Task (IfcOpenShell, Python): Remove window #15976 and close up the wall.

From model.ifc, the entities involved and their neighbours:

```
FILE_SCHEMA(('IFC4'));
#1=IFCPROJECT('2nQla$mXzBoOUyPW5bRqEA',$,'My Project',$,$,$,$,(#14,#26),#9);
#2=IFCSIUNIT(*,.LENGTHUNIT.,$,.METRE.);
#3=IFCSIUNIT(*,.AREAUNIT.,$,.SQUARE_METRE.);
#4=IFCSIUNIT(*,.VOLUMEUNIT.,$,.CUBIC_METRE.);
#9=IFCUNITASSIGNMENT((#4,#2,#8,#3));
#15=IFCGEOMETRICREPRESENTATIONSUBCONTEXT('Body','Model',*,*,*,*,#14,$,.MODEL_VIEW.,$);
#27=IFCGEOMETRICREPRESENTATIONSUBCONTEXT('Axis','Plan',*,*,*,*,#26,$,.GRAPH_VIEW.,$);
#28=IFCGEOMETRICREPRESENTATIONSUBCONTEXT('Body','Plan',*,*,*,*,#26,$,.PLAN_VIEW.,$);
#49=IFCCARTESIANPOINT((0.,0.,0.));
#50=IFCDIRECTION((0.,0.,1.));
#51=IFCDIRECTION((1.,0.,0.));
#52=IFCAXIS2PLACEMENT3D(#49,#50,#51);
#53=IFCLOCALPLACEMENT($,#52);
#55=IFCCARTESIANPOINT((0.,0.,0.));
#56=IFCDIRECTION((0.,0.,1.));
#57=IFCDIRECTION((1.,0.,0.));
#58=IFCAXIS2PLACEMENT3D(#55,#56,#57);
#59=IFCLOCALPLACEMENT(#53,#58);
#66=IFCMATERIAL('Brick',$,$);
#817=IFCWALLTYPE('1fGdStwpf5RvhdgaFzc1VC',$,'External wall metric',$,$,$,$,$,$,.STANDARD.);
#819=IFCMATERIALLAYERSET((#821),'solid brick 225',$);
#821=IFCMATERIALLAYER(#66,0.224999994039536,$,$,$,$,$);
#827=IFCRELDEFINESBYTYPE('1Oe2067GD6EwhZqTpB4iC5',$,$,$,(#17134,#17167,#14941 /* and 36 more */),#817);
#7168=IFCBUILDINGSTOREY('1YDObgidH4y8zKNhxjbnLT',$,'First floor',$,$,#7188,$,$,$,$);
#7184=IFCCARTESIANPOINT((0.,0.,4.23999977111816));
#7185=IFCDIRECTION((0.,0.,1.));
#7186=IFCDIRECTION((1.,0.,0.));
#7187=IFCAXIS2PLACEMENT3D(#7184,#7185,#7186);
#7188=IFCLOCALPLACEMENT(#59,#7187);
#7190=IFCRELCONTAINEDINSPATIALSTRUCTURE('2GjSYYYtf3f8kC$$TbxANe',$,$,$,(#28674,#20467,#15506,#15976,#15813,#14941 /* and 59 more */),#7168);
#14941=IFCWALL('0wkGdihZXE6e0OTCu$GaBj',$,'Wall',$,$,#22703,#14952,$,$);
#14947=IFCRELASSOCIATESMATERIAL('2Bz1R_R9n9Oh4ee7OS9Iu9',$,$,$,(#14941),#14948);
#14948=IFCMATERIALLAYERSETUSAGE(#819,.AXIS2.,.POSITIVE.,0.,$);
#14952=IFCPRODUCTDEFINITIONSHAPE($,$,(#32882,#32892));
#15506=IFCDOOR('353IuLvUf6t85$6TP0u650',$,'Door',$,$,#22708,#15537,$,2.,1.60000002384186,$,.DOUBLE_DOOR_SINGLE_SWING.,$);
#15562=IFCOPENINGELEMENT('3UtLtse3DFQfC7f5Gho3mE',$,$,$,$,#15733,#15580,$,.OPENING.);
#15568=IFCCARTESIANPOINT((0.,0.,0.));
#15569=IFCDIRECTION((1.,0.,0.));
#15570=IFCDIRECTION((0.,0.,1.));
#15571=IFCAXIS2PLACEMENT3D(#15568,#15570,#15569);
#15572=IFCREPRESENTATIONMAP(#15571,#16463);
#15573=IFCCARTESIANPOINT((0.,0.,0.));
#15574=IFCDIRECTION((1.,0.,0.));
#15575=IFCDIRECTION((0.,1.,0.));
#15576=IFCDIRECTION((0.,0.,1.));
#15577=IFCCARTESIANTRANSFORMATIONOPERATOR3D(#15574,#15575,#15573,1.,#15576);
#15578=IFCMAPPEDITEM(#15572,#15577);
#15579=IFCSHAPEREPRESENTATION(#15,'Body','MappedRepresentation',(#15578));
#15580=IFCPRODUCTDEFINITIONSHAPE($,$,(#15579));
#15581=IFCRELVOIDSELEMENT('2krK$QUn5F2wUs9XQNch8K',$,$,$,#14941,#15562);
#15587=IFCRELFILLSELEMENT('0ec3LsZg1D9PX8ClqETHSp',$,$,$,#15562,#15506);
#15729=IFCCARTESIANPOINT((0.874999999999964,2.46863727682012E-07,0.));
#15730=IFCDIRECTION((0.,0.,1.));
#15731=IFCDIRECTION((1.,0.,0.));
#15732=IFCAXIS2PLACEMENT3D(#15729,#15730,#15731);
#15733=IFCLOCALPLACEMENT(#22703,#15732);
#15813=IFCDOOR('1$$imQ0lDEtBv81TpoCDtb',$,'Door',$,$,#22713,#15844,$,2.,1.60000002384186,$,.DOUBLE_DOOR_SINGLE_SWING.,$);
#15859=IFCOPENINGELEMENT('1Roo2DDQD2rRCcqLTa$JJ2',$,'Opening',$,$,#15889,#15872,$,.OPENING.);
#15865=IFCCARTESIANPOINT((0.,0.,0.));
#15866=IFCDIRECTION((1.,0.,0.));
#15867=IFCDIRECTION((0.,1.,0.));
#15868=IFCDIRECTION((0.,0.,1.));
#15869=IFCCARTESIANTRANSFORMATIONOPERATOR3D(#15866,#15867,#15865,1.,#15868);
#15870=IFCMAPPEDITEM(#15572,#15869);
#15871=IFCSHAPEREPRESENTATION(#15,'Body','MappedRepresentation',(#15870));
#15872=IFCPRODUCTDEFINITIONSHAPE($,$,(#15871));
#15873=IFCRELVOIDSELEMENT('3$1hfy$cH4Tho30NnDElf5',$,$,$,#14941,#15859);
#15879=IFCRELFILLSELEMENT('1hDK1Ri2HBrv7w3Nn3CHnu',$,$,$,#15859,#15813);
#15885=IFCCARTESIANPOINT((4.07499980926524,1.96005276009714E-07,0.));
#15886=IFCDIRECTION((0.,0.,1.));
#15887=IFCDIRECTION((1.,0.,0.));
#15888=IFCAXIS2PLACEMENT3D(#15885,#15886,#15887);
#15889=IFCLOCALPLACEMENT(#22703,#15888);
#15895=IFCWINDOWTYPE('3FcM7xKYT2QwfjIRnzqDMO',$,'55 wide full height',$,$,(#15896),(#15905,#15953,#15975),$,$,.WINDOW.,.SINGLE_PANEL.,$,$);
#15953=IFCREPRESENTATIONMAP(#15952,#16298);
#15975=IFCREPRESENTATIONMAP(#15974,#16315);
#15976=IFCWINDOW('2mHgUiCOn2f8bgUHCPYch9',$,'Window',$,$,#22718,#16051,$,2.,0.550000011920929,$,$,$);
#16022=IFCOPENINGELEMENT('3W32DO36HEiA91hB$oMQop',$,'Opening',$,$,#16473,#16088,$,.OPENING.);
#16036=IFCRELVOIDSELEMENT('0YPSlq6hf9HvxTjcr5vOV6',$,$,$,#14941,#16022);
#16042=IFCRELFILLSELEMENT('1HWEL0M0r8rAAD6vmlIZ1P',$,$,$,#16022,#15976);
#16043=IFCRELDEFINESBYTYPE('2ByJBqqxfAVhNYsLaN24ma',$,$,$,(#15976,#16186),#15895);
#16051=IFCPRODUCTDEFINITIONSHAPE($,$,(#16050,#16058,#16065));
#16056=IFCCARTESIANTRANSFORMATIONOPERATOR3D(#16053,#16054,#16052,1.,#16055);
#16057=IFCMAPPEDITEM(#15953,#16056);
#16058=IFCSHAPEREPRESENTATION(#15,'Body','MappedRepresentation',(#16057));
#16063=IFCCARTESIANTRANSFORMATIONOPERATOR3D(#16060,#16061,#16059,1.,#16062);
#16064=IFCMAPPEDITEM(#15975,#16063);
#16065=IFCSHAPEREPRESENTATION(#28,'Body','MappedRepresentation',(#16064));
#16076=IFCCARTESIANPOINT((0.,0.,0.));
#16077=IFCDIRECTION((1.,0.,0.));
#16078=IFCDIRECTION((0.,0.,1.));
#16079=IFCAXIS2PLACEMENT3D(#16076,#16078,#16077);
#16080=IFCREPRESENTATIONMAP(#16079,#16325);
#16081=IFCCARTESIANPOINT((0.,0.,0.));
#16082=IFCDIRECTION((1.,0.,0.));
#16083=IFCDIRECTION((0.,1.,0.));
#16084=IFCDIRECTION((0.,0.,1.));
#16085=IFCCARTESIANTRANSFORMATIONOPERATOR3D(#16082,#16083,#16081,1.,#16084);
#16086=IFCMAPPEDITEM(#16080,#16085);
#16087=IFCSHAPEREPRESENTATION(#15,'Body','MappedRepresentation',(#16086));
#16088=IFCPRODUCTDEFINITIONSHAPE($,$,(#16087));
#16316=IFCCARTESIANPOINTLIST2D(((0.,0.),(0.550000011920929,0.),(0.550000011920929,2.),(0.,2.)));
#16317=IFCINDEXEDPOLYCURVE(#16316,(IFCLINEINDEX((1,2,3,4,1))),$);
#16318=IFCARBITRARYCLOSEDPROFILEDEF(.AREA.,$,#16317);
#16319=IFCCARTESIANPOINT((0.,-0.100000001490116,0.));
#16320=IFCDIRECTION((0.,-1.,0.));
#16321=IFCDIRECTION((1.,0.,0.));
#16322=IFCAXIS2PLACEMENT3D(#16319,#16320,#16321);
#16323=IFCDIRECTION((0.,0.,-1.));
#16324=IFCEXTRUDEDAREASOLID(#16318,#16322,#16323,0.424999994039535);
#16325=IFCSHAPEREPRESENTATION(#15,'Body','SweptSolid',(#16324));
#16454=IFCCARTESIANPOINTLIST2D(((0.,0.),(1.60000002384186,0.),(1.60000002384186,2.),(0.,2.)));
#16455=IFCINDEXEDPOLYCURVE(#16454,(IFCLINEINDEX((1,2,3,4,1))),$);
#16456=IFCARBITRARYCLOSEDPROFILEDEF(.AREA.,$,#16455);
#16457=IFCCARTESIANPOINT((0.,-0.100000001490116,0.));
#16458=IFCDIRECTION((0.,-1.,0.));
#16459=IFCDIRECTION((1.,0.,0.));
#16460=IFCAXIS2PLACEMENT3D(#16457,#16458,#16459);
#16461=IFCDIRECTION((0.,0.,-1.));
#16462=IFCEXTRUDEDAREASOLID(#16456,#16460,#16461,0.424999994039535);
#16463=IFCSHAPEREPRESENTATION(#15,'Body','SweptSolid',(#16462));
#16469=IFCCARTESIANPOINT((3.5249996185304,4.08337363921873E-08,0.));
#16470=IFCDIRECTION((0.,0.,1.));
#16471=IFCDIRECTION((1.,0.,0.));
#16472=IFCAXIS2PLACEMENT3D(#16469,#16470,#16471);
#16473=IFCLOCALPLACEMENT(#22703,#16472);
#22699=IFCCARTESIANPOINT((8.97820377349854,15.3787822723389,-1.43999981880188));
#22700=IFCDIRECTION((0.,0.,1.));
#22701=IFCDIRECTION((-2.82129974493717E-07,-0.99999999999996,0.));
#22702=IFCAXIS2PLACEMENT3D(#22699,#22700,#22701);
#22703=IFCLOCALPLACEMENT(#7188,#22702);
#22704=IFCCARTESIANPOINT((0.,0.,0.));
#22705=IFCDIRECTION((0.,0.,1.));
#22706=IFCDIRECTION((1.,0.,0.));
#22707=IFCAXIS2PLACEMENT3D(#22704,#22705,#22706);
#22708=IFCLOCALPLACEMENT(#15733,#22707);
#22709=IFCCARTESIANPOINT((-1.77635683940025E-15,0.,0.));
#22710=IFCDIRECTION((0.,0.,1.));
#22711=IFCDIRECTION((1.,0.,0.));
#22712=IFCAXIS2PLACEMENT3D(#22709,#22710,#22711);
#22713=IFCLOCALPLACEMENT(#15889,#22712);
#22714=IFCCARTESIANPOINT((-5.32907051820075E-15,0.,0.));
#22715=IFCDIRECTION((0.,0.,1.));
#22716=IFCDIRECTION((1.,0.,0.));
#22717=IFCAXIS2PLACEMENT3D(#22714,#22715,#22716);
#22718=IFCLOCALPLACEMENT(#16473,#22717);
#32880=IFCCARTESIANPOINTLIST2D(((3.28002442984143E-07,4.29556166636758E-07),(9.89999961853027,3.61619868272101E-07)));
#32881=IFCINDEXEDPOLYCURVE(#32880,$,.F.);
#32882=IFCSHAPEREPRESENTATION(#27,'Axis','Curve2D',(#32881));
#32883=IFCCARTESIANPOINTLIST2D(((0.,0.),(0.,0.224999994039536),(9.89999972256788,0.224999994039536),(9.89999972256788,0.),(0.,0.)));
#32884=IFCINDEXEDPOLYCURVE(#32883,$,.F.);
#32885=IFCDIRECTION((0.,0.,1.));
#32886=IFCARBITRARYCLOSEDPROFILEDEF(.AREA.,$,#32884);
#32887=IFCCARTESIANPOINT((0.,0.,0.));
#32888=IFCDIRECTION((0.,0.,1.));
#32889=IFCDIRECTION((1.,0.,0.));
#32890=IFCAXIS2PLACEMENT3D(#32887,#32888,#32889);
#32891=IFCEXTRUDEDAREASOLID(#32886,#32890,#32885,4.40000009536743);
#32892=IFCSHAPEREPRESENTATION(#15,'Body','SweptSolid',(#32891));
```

```python
import ifcopenshell
import ifcopenshell.api.feature
import ifcopenshell.api.root
import ifcopenshell.geom
import ifcopenshell.util.shape

model = ifcopenshell.open("model.ifc")
settings = ifcopenshell.geom.settings()


def volume(element):
    """Net volume in cubic metres, openings subtracted."""
    shape = ifcopenshell.geom.create_shape(settings, element)
    return ifcopenshell.util.shape.get_volume(shape.geometry)


window = model.by_guid("2mHgUiCOn2f8bgUHCPYch9")
opening = window.FillsVoids[0].RelatingOpeningElement
wall = opening.VoidsElements[0].RelatingBuildingElement
before = volume(wall)

ifcopenshell.api.root.remove_product(model, product=window)
ifcopenshell.api.feature.remove_feature(model, feature=opening)

after = volume(wall)

print(f"wall volume {before:.3f} -> {after:.3f} m3")

model.write("model_updated.ifc")
```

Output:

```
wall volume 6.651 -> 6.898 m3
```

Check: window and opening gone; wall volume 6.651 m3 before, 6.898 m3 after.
